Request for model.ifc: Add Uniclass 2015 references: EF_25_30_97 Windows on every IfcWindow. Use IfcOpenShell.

First a look at what the model holds.

```python
import ifcopenshell

model = ifcopenshell.open("model.ifc")
print(model.schema)
print("classifications:", [c.Name for c in model.by_type("IfcClassification")])
for ifc_class in ("IfcDoor", "IfcRoof", "IfcStair", "IfcWall", "IfcWindow"):
    print(ifc_class, len(model.by_type(ifc_class)))
```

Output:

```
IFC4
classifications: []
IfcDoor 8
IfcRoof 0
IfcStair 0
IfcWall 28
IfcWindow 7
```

```python
import ifcopenshell
import ifcopenshell.api.classification

model = ifcopenshell.open("model.ifc")

system = ifcopenshell.api.classification.add_classification(model, classification="Uniclass 2015")

codes = {
    "IfcWindow": ("EF_25_30_97", "Windows"),
}
for ifc_class, (code, name) in codes.items():
    products = model.by_type(ifc_class)
    ifcopenshell.api.classification.add_reference(
        model, products=products, classification=system, identification=code, name=name
    )
    print(code, len(products))

model.write("model_rev.ifc")
```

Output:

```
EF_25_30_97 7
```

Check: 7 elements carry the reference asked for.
